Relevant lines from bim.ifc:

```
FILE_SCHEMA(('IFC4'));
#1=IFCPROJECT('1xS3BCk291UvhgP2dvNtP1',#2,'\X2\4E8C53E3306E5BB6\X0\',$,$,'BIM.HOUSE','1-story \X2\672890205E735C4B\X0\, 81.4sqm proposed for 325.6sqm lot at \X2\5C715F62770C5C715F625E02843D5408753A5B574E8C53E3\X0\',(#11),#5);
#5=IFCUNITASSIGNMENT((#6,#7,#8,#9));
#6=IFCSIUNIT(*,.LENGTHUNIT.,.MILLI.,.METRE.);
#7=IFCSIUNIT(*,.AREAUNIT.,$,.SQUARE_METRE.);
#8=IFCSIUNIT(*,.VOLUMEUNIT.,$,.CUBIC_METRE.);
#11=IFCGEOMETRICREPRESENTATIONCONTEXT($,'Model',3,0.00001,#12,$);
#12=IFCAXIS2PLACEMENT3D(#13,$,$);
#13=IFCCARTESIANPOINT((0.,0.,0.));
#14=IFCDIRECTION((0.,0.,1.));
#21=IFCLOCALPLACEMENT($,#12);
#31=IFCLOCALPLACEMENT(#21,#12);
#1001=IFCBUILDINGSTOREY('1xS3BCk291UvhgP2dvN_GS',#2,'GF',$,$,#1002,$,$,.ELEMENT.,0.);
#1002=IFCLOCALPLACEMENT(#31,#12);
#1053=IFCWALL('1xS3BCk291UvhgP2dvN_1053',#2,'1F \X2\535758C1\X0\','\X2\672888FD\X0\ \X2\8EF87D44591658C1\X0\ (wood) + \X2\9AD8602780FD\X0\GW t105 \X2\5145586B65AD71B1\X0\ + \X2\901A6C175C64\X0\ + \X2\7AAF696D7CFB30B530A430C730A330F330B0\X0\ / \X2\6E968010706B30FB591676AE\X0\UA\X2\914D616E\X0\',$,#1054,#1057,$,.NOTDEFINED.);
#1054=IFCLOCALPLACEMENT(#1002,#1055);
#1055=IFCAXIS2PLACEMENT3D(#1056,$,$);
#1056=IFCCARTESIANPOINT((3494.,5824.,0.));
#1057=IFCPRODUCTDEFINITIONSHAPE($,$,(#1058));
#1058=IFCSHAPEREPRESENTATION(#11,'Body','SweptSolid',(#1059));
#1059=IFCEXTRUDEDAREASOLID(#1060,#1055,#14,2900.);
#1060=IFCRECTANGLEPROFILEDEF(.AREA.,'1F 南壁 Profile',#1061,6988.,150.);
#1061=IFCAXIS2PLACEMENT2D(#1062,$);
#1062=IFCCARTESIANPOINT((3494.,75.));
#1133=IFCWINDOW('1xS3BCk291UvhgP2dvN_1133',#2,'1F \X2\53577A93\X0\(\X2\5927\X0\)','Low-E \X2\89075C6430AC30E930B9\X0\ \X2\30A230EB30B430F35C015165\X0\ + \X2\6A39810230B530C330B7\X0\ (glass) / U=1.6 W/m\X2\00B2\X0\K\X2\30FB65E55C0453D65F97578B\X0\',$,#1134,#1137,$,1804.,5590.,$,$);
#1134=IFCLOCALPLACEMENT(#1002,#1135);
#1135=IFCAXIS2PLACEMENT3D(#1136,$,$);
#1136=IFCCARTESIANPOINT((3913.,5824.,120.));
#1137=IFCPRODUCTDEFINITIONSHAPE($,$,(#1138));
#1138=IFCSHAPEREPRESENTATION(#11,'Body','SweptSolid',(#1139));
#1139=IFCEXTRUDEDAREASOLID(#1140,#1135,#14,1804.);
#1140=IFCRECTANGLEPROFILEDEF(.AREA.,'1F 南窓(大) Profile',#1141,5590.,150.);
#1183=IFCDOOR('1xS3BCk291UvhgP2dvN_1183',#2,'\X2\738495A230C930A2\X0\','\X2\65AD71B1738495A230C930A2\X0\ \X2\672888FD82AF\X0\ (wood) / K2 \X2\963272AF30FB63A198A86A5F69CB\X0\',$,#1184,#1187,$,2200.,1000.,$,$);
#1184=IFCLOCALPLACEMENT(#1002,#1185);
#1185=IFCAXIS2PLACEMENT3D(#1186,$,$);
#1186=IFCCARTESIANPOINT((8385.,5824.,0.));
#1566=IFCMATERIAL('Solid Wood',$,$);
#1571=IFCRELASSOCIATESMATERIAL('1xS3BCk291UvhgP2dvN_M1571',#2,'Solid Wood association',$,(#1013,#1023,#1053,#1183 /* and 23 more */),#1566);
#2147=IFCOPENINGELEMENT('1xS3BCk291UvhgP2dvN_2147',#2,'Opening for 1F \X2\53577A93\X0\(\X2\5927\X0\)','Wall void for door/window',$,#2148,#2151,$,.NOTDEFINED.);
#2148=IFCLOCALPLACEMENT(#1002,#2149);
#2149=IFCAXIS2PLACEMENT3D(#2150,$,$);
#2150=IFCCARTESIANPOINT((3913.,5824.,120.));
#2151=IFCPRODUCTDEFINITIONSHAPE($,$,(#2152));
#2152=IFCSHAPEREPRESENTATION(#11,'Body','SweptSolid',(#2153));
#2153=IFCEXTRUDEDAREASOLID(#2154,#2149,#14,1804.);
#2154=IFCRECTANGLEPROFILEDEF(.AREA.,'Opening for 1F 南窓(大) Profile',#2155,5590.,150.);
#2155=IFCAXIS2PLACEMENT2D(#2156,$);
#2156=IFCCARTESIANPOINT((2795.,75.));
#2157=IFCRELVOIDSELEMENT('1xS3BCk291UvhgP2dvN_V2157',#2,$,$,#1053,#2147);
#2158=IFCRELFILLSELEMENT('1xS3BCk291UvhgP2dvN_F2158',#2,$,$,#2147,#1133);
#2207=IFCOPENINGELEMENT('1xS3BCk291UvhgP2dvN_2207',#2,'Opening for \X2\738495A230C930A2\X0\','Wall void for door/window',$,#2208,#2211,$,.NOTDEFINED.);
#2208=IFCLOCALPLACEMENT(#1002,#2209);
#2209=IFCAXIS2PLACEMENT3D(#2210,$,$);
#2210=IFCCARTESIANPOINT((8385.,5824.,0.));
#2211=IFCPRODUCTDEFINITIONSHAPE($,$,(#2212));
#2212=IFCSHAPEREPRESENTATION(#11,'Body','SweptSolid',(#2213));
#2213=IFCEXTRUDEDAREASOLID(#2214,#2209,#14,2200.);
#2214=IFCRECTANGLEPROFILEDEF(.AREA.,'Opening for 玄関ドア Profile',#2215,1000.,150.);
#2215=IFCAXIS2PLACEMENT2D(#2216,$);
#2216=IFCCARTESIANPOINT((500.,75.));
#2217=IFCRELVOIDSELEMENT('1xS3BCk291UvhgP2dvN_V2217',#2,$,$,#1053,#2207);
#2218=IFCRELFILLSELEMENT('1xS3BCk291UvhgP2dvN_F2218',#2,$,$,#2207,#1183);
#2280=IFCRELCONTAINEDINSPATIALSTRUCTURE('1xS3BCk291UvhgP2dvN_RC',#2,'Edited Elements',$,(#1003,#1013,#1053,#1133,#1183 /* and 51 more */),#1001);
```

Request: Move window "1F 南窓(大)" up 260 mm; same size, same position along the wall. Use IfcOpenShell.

```python
import numpy as np
import ifcopenshell
import ifcopenshell.api.geometry
import ifcopenshell.util.placement
import ifcopenshell.util.unit

model = ifcopenshell.open("bim.ifc")
unit_scale = ifcopenshell.util.unit.calculate_unit_scale(model)

window = model.by_guid("1xS3BCk291UvhgP2dvN_1133")
opening = window.FillsVoids[0].RelatingOpeningElement
dz = 0.26 / unit_scale

shift = np.array([0.0, 0.0, dz])
# The window is not placed relative to its opening, so move both.
for product in (opening, window):
    matrix = ifcopenshell.util.placement.get_local_placement(product.ObjectPlacement)
    matrix[:3, 3] += shift
    ifcopenshell.api.geometry.edit_object_placement(model, product=product, matrix=matrix, is_si=False)

print(f"moved by {dz * unit_scale:+.3f} m")

model.write("bim_v2.ifc")
```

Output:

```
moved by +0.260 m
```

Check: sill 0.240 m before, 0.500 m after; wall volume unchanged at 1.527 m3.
